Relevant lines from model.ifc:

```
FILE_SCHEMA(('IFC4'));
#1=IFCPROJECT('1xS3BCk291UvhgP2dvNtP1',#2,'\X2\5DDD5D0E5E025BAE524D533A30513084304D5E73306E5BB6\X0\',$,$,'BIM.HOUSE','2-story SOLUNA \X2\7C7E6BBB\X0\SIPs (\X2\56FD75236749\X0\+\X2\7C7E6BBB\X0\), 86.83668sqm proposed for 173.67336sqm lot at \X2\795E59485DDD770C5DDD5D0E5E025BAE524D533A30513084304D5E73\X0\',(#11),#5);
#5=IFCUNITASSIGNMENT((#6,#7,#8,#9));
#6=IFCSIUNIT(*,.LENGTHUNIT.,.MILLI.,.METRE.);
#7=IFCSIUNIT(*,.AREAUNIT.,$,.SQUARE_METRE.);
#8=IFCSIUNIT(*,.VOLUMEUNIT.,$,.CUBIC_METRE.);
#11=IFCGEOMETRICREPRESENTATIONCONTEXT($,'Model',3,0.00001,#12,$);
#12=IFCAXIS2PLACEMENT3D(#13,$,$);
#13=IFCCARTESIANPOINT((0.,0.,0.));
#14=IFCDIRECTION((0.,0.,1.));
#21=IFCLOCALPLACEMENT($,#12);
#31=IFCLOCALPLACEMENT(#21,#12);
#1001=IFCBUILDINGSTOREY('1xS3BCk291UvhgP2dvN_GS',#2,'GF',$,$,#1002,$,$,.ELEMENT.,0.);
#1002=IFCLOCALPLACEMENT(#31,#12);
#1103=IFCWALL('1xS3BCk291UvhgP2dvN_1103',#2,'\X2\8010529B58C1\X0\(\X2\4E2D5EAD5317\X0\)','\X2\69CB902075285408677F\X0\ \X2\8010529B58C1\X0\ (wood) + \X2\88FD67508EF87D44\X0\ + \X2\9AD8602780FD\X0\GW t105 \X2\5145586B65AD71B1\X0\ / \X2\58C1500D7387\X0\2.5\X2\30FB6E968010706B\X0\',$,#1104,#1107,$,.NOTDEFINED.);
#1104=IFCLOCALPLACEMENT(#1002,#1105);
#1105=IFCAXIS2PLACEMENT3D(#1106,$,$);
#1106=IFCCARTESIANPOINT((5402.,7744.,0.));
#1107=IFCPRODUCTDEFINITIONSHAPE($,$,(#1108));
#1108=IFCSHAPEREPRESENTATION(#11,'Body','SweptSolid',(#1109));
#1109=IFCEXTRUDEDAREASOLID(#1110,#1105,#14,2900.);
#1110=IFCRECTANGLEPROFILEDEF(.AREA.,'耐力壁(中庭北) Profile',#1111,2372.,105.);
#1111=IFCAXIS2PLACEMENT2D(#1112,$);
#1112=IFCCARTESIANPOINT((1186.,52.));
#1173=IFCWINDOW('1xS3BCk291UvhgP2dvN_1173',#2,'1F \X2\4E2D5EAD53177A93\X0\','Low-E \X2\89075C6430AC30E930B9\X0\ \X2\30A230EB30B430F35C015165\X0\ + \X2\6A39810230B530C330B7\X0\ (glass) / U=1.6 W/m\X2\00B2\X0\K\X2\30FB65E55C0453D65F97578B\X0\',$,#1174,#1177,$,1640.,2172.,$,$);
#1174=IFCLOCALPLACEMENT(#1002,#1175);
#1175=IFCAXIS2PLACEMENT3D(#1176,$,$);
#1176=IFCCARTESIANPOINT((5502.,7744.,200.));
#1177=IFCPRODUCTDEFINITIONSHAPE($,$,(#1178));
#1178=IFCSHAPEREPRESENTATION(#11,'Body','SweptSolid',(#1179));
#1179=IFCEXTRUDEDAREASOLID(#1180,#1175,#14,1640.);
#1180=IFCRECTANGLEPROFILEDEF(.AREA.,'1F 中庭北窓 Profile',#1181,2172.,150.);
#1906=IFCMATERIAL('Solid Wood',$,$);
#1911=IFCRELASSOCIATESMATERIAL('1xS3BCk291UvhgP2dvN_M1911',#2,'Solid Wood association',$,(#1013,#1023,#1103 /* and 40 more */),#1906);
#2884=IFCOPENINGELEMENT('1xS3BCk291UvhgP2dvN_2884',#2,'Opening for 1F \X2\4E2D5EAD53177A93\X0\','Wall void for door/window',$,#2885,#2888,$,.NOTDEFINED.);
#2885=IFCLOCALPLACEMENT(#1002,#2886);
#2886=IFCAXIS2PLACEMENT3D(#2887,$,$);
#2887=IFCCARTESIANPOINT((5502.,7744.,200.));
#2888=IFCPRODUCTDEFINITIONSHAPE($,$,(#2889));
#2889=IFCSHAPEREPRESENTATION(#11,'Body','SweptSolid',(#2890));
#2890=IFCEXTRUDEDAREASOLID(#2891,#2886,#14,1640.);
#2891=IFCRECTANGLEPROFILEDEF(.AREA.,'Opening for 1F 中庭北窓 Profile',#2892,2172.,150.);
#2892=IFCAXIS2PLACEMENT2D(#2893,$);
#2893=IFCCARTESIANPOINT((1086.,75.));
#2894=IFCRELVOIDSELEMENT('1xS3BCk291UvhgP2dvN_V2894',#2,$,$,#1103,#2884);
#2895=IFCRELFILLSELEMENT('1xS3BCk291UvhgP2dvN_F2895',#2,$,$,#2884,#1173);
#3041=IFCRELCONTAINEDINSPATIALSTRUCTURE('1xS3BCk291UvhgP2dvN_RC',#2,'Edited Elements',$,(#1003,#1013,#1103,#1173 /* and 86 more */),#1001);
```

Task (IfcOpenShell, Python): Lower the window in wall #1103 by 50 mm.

```python
import numpy as np
import ifcopenshell
import ifcopenshell.api.geometry
import ifcopenshell.util.placement
import ifcopenshell.util.unit

model = ifcopenshell.open("model.ifc")
unit_scale = ifcopenshell.util.unit.calculate_unit_scale(model)

window = model.by_guid("1xS3BCk291UvhgP2dvN_1173")
opening = window.FillsVoids[0].RelatingOpeningElement
dz = -50.0

shift = np.array([0.0, 0.0, dz])
# The window is not placed relative to its opening, so move both.
for product in (opening, window):
    matrix = ifcopenshell.util.placement.get_local_placement(product.ObjectPlacement)
    matrix[:3, 3] += shift
    ifcopenshell.api.geometry.edit_object_placement(model, product=product, matrix=matrix, is_si=False)

print(f"moved by {dz * unit_scale:+.3f} m")

model.write("model_updated.ifc")
```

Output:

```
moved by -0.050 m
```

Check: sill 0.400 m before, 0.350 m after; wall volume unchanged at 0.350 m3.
